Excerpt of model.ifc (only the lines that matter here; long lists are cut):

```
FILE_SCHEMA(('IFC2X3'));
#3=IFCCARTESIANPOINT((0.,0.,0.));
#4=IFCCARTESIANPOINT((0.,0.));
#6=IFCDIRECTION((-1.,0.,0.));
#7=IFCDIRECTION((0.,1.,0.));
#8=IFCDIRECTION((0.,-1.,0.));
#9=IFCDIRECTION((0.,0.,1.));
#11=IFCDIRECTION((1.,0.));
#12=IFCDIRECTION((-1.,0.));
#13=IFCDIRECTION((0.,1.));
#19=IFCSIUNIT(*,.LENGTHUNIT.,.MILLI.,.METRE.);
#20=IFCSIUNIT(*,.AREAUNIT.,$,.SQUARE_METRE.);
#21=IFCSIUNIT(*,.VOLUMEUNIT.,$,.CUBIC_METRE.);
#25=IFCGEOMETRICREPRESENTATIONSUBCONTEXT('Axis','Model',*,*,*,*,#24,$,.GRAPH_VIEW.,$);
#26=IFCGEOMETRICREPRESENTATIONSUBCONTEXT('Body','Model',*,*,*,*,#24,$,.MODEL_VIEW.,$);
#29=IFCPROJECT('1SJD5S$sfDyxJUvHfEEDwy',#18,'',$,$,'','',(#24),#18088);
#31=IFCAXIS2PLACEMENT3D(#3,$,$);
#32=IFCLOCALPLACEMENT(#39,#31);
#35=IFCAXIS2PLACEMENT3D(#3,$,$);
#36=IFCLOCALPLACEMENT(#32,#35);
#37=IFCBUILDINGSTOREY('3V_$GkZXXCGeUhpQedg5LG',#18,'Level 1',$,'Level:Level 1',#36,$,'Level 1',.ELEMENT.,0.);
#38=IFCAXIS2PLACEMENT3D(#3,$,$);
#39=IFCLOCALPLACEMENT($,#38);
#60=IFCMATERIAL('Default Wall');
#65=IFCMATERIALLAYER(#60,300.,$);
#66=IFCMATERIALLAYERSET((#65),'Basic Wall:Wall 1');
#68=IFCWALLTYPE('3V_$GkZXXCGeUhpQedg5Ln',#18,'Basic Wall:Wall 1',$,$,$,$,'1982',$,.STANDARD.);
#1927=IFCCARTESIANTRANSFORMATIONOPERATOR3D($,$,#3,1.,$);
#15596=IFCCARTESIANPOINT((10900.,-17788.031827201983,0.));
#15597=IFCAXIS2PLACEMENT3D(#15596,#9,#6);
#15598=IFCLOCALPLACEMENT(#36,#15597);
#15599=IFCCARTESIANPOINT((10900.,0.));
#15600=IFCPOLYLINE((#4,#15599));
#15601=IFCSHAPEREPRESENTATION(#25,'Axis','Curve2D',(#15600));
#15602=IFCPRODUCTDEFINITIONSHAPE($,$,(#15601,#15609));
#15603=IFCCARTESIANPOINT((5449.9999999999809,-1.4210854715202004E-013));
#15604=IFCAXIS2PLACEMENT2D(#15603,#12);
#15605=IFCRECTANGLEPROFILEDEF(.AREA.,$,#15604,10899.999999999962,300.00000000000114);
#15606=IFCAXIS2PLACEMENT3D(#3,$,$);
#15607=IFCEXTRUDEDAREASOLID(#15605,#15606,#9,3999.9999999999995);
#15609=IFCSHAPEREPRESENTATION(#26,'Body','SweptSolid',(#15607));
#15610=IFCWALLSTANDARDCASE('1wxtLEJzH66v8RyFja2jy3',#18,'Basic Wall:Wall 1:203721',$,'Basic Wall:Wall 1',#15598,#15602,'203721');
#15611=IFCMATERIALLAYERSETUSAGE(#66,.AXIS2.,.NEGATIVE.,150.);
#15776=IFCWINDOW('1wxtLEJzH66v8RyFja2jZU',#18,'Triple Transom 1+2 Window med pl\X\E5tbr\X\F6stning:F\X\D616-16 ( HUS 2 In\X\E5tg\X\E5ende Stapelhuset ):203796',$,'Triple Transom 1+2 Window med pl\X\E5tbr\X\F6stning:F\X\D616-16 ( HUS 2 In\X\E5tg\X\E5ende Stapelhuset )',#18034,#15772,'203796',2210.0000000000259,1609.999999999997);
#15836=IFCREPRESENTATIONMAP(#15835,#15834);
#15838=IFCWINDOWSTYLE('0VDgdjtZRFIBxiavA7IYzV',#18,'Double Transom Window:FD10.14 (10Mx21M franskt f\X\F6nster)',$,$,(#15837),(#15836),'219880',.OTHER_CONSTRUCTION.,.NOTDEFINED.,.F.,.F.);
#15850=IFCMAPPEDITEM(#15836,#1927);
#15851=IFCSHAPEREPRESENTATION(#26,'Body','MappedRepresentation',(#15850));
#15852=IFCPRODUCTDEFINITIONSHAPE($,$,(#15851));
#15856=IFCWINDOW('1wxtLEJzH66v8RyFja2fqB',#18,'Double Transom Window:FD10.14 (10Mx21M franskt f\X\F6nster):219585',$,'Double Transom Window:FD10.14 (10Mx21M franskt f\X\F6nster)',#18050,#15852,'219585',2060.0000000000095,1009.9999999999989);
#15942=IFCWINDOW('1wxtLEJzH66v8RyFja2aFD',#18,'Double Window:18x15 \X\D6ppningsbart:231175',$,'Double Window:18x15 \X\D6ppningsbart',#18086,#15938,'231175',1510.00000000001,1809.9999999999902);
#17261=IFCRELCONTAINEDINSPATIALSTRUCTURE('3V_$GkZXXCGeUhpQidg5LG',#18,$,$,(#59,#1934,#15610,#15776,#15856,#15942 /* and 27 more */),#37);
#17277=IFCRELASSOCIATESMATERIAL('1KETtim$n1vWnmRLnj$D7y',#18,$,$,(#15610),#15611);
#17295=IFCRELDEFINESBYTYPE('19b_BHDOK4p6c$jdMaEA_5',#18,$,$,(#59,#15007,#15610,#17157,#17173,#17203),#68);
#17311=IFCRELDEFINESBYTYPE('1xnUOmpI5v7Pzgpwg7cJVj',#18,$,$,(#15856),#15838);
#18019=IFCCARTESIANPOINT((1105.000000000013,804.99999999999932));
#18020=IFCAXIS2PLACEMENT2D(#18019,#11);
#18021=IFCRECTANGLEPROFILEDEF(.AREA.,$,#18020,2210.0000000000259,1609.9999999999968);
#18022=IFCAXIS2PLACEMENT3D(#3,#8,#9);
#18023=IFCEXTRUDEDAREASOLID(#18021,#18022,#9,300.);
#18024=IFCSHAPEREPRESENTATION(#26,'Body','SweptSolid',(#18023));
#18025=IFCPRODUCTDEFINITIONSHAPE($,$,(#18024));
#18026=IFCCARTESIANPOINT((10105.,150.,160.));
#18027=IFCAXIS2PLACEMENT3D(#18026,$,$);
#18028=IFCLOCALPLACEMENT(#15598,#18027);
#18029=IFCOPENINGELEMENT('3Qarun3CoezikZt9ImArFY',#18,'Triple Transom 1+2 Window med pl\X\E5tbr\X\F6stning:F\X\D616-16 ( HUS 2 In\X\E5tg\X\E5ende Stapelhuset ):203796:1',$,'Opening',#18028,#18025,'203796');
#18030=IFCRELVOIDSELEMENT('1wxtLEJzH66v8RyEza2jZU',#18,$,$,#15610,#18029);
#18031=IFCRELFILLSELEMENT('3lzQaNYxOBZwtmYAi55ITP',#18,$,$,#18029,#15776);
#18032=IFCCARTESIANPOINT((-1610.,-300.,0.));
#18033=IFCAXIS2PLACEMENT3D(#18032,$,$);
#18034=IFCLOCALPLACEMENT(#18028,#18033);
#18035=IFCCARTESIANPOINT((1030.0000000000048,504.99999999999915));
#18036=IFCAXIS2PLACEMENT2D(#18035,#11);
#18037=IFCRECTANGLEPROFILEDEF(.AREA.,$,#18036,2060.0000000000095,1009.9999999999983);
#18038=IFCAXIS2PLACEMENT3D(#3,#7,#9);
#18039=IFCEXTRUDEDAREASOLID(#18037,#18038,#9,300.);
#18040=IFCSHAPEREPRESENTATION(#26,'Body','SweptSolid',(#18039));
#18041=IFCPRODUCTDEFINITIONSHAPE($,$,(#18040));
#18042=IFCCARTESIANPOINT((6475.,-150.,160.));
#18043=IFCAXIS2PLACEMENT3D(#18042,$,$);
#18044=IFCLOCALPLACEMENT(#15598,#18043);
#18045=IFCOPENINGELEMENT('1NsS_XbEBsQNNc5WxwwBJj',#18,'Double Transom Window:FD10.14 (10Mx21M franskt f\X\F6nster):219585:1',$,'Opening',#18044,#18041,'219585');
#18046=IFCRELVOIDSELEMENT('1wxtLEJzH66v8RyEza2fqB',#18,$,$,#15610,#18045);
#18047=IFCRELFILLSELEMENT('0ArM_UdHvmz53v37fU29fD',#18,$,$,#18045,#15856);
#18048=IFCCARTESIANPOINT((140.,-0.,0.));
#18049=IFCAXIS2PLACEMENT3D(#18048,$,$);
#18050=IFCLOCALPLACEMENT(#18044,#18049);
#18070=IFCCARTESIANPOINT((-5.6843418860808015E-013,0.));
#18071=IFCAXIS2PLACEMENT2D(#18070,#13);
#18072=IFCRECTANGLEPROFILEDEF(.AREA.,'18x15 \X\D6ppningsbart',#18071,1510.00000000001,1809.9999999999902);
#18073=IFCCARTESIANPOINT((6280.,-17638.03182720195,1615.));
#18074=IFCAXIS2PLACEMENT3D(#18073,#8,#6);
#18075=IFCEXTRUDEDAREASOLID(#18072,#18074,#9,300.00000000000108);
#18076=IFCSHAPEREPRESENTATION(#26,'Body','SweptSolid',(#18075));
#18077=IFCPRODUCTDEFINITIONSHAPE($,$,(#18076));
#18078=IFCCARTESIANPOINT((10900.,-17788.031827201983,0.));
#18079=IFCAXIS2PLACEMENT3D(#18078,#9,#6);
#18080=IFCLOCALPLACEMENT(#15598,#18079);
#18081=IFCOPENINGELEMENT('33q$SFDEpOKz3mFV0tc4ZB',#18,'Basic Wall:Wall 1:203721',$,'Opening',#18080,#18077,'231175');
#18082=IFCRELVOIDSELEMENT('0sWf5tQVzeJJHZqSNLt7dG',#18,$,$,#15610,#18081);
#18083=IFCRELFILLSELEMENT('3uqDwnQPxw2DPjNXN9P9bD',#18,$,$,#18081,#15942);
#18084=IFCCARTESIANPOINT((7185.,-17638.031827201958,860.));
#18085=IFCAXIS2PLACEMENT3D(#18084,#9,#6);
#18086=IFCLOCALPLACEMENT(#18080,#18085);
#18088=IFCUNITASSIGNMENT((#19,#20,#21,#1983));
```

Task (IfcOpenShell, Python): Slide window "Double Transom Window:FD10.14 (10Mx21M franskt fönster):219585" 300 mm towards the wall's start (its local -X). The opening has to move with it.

```python
import ifcopenshell
import ifcopenshell.api.geometry
import ifcopenshell.util.placement

model = ifcopenshell.open("model.ifc")

window = model.by_id(15856)
opening = window.FillsVoids[0].RelatingOpeningElement
wall = opening.VoidsElements[0].RelatingBuildingElement

wall_matrix = ifcopenshell.util.placement.get_local_placement(wall.ObjectPlacement)
shift = wall_matrix[:3, 0] * -300.0
before = ifcopenshell.util.placement.get_local_placement(window.ObjectPlacement)[:3, 3].copy()

# The window is placed relative to its opening, so it follows when the opening moves.
matrix = ifcopenshell.util.placement.get_local_placement(opening.ObjectPlacement)
matrix[:3, 3] += shift
ifcopenshell.api.geometry.edit_object_placement(
    model, product=opening, matrix=matrix, is_si=False, should_transform_children=True
)

after = ifcopenshell.util.placement.get_local_placement(window.ObjectPlacement)[:3, 3]
print("window moved by", (after - before).round(3) + 0.0)

model.write("model_updated.ifc")
```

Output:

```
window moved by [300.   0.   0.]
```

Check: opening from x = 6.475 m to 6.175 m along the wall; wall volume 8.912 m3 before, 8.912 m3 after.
